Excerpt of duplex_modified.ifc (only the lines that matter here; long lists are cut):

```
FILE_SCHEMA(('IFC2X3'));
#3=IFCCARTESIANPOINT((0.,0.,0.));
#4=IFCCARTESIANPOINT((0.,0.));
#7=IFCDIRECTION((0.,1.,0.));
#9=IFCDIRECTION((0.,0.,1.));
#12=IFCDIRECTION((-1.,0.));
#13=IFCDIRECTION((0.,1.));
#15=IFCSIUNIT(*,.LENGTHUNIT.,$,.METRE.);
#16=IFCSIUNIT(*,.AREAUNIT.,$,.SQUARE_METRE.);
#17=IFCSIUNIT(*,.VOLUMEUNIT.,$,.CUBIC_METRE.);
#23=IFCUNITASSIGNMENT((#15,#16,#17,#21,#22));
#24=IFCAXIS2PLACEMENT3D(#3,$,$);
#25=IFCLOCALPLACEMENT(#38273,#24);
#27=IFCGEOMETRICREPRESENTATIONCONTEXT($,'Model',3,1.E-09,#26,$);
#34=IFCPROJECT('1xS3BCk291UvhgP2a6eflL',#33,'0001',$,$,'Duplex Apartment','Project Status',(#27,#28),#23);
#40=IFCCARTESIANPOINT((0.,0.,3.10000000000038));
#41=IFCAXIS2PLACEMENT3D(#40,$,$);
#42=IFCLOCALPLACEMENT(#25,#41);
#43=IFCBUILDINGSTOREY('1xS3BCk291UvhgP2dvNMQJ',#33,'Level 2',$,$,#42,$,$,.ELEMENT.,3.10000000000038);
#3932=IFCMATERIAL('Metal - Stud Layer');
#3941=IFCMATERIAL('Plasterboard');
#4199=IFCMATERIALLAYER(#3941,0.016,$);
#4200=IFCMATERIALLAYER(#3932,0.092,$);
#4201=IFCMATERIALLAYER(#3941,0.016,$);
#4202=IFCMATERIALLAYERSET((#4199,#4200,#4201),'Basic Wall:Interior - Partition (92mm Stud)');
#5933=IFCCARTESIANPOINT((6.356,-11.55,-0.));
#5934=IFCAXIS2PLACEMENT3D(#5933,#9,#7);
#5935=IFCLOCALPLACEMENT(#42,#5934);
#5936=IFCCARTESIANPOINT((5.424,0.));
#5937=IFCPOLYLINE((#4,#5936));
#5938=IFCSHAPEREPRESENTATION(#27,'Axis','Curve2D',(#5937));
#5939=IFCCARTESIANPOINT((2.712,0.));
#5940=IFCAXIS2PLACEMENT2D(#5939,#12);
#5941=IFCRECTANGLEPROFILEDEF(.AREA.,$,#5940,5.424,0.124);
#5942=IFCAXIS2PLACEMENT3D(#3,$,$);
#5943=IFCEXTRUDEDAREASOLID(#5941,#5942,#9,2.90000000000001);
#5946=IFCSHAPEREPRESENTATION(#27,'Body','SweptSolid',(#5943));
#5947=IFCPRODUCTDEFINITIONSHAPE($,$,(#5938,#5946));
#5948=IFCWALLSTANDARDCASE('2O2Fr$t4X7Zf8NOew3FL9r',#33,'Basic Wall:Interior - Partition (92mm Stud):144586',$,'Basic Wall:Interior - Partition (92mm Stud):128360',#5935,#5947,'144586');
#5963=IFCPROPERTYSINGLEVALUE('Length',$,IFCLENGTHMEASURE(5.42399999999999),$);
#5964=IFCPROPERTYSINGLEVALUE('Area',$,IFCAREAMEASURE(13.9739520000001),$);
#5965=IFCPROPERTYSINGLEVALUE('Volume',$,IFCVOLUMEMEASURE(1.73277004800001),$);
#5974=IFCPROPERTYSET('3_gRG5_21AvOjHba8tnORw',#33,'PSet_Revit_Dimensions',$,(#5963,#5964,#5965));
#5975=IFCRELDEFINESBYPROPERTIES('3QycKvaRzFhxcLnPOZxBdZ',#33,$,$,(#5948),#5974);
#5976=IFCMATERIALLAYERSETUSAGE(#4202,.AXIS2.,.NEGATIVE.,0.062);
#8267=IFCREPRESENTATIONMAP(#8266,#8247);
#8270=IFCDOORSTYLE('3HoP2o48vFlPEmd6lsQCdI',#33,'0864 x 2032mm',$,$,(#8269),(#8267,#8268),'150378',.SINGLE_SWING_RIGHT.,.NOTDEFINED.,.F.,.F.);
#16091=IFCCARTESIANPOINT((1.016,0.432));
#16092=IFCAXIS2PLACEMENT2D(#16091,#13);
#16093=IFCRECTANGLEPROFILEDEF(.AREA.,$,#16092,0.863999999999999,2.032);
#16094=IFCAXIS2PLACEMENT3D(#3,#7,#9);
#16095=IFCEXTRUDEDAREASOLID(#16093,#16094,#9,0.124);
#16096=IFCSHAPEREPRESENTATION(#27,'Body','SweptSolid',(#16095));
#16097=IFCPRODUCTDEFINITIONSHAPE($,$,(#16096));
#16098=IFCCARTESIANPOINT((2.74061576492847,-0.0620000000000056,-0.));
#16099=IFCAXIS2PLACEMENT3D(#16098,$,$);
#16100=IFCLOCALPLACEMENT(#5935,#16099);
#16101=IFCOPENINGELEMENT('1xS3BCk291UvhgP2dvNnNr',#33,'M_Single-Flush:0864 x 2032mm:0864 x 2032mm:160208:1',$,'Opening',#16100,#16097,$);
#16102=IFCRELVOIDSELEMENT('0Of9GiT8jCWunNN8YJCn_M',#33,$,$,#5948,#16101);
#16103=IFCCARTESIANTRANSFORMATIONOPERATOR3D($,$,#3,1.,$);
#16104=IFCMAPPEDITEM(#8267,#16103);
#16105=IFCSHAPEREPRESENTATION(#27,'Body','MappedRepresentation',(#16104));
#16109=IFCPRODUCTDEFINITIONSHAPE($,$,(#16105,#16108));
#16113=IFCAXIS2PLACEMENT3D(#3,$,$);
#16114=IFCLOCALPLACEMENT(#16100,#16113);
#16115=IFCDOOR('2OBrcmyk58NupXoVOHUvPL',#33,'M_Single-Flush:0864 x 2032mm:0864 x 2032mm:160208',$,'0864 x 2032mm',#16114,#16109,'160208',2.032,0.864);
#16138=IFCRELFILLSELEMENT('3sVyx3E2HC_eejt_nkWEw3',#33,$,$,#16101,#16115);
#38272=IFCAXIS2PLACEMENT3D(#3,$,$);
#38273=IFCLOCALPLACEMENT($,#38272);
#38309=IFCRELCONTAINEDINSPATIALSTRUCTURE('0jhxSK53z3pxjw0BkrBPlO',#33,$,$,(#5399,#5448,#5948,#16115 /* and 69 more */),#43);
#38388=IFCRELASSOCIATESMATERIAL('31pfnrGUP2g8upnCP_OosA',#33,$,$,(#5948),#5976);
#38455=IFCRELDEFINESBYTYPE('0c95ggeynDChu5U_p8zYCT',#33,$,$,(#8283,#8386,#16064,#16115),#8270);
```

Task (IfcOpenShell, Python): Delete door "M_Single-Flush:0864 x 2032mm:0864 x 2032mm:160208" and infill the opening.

```python
import ifcopenshell
import ifcopenshell.api.feature
import ifcopenshell.api.pset
import ifcopenshell.api.root
import ifcopenshell.geom
import ifcopenshell.util.element
import ifcopenshell.util.shape
import ifcopenshell.util.unit

model = ifcopenshell.open("duplex_modified.ifc")
area_scale = ifcopenshell.util.unit.calculate_unit_scale(model, "AREAUNIT")
volume_scale = ifcopenshell.util.unit.calculate_unit_scale(model, "VOLUMEUNIT")
settings = ifcopenshell.geom.settings()


def volume(element):
    """Net volume in cubic metres, openings subtracted."""
    shape = ifcopenshell.geom.create_shape(settings, element)
    return ifcopenshell.util.shape.get_volume(shape.geometry)


door = model.by_guid("2OBrcmyk58NupXoVOHUvPL")
opening = door.FillsVoids[0].RelatingOpeningElement
wall = opening.VoidsElements[0].RelatingBuildingElement
before = volume(wall)

ifcopenshell.api.root.remove_product(model, product=door)
ifcopenshell.api.feature.remove_feature(model, feature=opening)

after = volume(wall)
thickness = 0.124  # wall thickness in metres

# Update the wall's stored quantities.
pset = model.by_id(ifcopenshell.util.element.get_pset(wall, "PSet_Revit_Dimensions", should_inherit=False)["id"])
ifcopenshell.api.pset.edit_pset(model, pset=pset, properties={
    "Area": model.create_entity("IfcAreaMeasure", after / thickness / area_scale),
    "Volume": model.create_entity("IfcVolumeMeasure", after / volume_scale),
})

print(f"wall volume {before:.3f} -> {after:.3f} m3")

model.write("duplex_modified-out.ifc")
```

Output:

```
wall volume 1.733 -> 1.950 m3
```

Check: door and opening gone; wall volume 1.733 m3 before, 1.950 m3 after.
